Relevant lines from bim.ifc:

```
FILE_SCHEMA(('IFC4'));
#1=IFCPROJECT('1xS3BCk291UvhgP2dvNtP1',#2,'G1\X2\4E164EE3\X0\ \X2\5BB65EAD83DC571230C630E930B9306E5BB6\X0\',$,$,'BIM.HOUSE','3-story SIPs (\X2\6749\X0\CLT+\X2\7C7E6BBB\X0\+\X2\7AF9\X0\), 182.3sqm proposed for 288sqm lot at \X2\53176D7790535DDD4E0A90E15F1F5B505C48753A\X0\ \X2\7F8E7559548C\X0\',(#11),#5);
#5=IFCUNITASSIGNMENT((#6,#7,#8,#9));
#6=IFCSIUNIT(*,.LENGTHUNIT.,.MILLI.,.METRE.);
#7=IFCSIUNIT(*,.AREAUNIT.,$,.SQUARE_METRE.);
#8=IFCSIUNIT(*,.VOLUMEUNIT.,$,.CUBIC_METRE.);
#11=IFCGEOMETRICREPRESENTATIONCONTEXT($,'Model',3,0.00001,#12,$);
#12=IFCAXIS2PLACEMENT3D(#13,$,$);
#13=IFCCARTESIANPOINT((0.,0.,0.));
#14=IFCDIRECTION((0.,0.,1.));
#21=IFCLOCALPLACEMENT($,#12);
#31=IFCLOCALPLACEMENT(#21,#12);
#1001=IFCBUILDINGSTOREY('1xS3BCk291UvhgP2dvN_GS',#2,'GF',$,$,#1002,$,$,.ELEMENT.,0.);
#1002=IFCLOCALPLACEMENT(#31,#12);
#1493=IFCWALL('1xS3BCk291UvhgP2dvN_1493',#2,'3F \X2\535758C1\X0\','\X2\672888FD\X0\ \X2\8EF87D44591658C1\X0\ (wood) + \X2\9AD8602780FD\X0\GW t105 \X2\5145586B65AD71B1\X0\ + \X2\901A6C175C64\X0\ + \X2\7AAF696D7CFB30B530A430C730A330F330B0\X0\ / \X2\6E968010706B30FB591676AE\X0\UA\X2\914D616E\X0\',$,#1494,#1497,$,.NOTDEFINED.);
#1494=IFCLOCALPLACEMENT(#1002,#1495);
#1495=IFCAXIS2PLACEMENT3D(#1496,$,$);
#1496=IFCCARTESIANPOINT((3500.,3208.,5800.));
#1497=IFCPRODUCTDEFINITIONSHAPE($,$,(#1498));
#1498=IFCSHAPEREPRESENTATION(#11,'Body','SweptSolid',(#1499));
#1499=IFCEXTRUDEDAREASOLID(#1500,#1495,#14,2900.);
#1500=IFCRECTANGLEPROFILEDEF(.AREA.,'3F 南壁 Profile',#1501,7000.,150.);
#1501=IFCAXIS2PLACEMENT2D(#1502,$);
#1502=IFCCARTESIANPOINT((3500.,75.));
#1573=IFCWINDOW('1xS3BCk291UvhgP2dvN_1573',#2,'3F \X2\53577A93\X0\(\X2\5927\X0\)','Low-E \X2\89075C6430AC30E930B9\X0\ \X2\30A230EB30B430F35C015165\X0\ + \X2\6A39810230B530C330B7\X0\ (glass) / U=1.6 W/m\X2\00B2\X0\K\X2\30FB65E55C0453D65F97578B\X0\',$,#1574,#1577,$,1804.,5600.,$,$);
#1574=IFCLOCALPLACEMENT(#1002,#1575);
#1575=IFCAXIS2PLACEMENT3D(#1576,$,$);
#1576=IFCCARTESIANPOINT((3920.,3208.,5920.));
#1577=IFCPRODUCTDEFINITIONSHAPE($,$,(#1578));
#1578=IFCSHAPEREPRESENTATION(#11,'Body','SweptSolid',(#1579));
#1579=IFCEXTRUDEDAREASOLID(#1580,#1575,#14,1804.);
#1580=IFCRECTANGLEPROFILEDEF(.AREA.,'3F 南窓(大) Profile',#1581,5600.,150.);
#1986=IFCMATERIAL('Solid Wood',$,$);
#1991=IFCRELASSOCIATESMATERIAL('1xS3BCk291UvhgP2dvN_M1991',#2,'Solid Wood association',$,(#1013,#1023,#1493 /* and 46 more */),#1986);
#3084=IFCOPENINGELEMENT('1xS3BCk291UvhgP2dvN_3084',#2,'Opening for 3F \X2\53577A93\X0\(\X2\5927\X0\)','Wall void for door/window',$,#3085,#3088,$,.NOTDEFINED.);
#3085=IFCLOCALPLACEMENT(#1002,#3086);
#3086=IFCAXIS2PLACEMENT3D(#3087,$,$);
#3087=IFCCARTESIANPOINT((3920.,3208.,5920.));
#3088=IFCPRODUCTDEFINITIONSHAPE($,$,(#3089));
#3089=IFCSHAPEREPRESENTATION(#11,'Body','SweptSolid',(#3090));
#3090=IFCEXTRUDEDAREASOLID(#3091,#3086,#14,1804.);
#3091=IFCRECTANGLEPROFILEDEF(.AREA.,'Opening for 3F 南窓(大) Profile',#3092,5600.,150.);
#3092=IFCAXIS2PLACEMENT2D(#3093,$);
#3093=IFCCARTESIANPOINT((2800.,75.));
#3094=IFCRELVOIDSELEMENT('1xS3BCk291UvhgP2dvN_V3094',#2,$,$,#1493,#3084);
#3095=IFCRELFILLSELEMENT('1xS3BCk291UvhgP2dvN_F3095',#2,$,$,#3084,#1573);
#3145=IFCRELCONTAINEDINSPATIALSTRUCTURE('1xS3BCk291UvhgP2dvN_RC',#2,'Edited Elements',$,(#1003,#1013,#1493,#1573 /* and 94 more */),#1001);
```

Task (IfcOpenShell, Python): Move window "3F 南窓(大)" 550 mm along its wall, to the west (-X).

```python
import ifcopenshell
import ifcopenshell.api.geometry
import ifcopenshell.util.placement

model = ifcopenshell.open("bim.ifc")

window = model.by_guid("1xS3BCk291UvhgP2dvN_1573")
opening = window.FillsVoids[0].RelatingOpeningElement
wall = opening.VoidsElements[0].RelatingBuildingElement

wall_matrix = ifcopenshell.util.placement.get_local_placement(wall.ObjectPlacement)
shift = wall_matrix[:3, 0] * -550.0
before = ifcopenshell.util.placement.get_local_placement(window.ObjectPlacement)[:3, 3].copy()

# The window is not placed relative to its opening, so move both.
for product in (opening, window):
    matrix = ifcopenshell.util.placement.get_local_placement(product.ObjectPlacement)
    matrix[:3, 3] += shift
    ifcopenshell.api.geometry.edit_object_placement(model, product=product, matrix=matrix, is_si=False)

after = ifcopenshell.util.placement.get_local_placement(window.ObjectPlacement)[:3, 3]
print("window moved by", (after - before).round(3) + 0.0)

model.write("bim_v2.ifc")
```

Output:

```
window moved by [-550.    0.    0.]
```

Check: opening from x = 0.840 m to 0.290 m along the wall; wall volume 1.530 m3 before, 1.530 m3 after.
